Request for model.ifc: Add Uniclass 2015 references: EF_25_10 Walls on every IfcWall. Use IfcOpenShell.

First a look at what the model holds.

```python
import ifcopenshell

model = ifcopenshell.open("model.ifc")
print(model.schema)
print("classifications:", [c.Name for c in model.by_type("IfcClassification")])
for ifc_class in ("IfcDoor", "IfcRoof", "IfcStair", "IfcWall", "IfcWindow"):
    print(ifc_class, len(model.by_type(ifc_class)))
```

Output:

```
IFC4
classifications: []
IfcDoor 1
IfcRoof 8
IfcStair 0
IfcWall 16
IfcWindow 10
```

```python
import ifcopenshell
import ifcopenshell.api.classification

model = ifcopenshell.open("model.ifc")

system = ifcopenshell.api.classification.add_classification(model, classification="Uniclass 2015")

codes = {
    "IfcWall": ("EF_25_10", "Walls"),
}
for ifc_class, (code, name) in codes.items():
    products = model.by_type(ifc_class)
    ifcopenshell.api.classification.add_reference(
        model, products=products, classification=system, identification=code, name=name
    )
    print(code, len(products))

model.write("model_edited.ifc")
```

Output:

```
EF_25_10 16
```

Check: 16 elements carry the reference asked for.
